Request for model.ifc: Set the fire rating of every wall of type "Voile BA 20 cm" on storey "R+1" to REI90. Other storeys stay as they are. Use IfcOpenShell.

First a look at what the model holds.

```python
import ifcopenshell
import ifcopenshell.util.element

model = ifcopenshell.open("model.ifc")
print(model.schema)
storey = next(s for s in model.by_type("IfcBuildingStorey") if s.Name == "R+1")
walls = [e for e in ifcopenshell.util.element.get_decomposition(storey) if e.is_a("IfcWall")]
seen = {}
for e in walls:
    element_type = ifcopenshell.util.element.get_type(e)
    key = (element_type.Name if element_type != e and element_type else None, ifcopenshell.util.element.get_pset(e, "Pset_WallCommon", "FireRating"))
    seen[key] = seen.get(key, 0) + 1
for (name, value), count in sorted(seen.items(), key=str):
    print(count, "x", name, "|", value)
```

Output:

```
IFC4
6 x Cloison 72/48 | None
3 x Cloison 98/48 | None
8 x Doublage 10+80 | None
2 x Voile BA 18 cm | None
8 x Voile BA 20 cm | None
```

```python
import ifcopenshell
import ifcopenshell.api.pset
import ifcopenshell.util.element

model = ifcopenshell.open("model.ifc")

storey = next(s for s in model.by_type("IfcBuildingStorey") if s.Name == "R+1")
walls = [e for e in ifcopenshell.util.element.get_decomposition(storey) if e.is_a("IfcWall")]

count = 0
for e in walls:
    element_type = ifcopenshell.util.element.get_type(e)
    if element_type in (None, e) or element_type.Name != "Voile BA 20 cm":
        continue
    # add_pset returns the element's existing set when there is one.
    pset = ifcopenshell.api.pset.add_pset(model, product=e, name="Pset_WallCommon")
    ifcopenshell.api.pset.edit_pset(model, pset=pset, properties={"FireRating": "REI90"})
    count += 1

print(count, "walls updated")

model.write("model_rev.ifc")
```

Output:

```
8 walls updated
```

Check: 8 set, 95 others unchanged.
